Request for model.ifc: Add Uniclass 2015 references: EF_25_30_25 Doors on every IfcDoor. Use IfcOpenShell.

First a look at what the model holds.

```python
import ifcopenshell

model = ifcopenshell.open("model.ifc")
print(model.schema)
print("classifications:", [c.Name for c in model.by_type("IfcClassification")])
for ifc_class in ("IfcDoor", "IfcRoof", "IfcStair", "IfcWall", "IfcWindow"):
    print(ifc_class, len(model.by_type(ifc_class)))
```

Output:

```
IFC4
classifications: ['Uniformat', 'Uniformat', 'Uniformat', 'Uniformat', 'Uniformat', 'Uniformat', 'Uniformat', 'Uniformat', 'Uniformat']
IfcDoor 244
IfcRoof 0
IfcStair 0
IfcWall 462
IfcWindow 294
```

```python
import ifcopenshell
import ifcopenshell.api.classification

model = ifcopenshell.open("model.ifc")

system = ifcopenshell.api.classification.add_classification(model, classification="Uniclass 2015")

codes = {
    "IfcDoor": ("EF_25_30_25", "Doors"),
}
for ifc_class, (code, name) in codes.items():
    products = model.by_type(ifc_class)
    ifcopenshell.api.classification.add_reference(
        model, products=products, classification=system, identification=code, name=name
    )
    print(code, len(products))

model.write("model-out.ifc")
```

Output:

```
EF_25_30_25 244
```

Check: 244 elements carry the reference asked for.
